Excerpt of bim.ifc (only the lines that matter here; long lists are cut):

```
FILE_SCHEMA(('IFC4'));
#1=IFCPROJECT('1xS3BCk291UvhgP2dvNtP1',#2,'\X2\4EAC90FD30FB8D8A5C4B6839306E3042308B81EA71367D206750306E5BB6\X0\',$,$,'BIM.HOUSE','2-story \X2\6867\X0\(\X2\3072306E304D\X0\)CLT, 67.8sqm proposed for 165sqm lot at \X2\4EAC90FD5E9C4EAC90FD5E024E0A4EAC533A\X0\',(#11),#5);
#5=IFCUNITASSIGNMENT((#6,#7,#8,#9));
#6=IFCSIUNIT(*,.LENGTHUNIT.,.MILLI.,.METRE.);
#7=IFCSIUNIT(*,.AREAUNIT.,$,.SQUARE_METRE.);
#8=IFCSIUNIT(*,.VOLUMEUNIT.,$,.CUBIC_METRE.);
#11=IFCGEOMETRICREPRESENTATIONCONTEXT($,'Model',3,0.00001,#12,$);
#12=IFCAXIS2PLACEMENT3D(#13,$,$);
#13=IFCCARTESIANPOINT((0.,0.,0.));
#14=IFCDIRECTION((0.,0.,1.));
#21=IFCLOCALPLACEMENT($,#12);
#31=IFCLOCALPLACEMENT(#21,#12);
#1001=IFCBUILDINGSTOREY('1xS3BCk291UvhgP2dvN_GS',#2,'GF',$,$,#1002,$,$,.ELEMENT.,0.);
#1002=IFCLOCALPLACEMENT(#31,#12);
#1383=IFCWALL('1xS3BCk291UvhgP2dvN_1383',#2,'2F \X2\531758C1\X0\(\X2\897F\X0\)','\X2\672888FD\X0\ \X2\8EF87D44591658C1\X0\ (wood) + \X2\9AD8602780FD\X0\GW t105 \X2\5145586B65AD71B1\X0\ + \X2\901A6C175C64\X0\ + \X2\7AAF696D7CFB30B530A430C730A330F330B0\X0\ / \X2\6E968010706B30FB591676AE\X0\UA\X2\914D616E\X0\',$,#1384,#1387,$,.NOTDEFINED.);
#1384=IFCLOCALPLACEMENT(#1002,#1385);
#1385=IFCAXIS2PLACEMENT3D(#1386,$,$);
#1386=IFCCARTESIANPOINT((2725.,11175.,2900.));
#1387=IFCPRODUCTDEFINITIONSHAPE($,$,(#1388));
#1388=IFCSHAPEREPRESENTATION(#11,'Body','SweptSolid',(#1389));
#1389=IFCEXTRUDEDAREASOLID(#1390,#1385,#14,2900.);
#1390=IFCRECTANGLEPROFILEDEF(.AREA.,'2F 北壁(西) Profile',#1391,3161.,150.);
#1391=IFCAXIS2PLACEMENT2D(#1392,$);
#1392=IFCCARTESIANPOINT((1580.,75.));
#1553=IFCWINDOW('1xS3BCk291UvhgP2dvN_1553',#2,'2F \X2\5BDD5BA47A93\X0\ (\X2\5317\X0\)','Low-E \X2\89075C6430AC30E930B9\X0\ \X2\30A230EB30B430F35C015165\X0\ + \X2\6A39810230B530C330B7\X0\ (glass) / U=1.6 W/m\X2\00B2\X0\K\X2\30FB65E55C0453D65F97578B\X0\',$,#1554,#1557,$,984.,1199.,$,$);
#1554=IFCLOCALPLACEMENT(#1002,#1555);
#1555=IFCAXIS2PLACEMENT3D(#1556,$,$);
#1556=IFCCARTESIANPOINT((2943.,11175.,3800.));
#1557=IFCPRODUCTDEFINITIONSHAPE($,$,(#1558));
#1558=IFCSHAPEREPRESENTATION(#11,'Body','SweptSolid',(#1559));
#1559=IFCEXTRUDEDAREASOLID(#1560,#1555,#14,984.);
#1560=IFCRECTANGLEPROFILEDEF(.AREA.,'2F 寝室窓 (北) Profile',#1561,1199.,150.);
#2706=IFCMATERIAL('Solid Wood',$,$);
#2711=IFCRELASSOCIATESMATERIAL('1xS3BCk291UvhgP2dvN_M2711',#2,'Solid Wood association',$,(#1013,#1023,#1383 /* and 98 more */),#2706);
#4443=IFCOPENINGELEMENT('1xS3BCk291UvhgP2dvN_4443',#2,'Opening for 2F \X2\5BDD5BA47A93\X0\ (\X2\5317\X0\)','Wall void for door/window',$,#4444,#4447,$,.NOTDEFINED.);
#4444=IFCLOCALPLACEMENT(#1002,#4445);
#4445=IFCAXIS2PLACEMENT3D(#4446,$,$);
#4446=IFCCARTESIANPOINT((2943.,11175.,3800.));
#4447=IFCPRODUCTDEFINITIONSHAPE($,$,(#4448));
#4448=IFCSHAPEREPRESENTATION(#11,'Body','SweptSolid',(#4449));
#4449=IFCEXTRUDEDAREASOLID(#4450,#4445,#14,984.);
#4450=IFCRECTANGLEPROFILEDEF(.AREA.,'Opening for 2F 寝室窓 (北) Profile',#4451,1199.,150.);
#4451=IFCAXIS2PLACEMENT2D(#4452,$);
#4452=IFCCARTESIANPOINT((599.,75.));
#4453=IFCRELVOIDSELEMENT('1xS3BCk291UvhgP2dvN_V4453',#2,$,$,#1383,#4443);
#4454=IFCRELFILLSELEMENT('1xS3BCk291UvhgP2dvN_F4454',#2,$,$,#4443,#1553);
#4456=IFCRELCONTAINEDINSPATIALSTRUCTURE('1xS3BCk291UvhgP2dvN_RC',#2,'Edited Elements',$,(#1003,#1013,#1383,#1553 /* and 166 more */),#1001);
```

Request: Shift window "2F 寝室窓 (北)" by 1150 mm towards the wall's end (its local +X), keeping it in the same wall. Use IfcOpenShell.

```python
import ifcopenshell
import ifcopenshell.api.geometry
import ifcopenshell.util.placement
import ifcopenshell.util.unit

model = ifcopenshell.open("bim.ifc")
unit_scale = ifcopenshell.util.unit.calculate_unit_scale(model)

window = model.by_guid("1xS3BCk291UvhgP2dvN_1553")
opening = window.FillsVoids[0].RelatingOpeningElement
wall = opening.VoidsElements[0].RelatingBuildingElement

wall_matrix = ifcopenshell.util.placement.get_local_placement(wall.ObjectPlacement)
shift = wall_matrix[:3, 0] * 1.15 / unit_scale
before = ifcopenshell.util.placement.get_local_placement(window.ObjectPlacement)[:3, 3].copy()

# The window is not placed relative to its opening, so move both.
for product in (opening, window):
    matrix = ifcopenshell.util.placement.get_local_placement(product.ObjectPlacement)
    matrix[:3, 3] += shift
    ifcopenshell.api.geometry.edit_object_placement(model, product=product, matrix=matrix, is_si=False)

after = ifcopenshell.util.placement.get_local_placement(window.ObjectPlacement)[:3, 3]
print("window moved by", (after - before).round(3) + 0.0)

model.write("bim_rev.ifc")
```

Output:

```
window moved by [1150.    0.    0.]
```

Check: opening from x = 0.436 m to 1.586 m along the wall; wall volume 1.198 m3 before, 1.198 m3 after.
